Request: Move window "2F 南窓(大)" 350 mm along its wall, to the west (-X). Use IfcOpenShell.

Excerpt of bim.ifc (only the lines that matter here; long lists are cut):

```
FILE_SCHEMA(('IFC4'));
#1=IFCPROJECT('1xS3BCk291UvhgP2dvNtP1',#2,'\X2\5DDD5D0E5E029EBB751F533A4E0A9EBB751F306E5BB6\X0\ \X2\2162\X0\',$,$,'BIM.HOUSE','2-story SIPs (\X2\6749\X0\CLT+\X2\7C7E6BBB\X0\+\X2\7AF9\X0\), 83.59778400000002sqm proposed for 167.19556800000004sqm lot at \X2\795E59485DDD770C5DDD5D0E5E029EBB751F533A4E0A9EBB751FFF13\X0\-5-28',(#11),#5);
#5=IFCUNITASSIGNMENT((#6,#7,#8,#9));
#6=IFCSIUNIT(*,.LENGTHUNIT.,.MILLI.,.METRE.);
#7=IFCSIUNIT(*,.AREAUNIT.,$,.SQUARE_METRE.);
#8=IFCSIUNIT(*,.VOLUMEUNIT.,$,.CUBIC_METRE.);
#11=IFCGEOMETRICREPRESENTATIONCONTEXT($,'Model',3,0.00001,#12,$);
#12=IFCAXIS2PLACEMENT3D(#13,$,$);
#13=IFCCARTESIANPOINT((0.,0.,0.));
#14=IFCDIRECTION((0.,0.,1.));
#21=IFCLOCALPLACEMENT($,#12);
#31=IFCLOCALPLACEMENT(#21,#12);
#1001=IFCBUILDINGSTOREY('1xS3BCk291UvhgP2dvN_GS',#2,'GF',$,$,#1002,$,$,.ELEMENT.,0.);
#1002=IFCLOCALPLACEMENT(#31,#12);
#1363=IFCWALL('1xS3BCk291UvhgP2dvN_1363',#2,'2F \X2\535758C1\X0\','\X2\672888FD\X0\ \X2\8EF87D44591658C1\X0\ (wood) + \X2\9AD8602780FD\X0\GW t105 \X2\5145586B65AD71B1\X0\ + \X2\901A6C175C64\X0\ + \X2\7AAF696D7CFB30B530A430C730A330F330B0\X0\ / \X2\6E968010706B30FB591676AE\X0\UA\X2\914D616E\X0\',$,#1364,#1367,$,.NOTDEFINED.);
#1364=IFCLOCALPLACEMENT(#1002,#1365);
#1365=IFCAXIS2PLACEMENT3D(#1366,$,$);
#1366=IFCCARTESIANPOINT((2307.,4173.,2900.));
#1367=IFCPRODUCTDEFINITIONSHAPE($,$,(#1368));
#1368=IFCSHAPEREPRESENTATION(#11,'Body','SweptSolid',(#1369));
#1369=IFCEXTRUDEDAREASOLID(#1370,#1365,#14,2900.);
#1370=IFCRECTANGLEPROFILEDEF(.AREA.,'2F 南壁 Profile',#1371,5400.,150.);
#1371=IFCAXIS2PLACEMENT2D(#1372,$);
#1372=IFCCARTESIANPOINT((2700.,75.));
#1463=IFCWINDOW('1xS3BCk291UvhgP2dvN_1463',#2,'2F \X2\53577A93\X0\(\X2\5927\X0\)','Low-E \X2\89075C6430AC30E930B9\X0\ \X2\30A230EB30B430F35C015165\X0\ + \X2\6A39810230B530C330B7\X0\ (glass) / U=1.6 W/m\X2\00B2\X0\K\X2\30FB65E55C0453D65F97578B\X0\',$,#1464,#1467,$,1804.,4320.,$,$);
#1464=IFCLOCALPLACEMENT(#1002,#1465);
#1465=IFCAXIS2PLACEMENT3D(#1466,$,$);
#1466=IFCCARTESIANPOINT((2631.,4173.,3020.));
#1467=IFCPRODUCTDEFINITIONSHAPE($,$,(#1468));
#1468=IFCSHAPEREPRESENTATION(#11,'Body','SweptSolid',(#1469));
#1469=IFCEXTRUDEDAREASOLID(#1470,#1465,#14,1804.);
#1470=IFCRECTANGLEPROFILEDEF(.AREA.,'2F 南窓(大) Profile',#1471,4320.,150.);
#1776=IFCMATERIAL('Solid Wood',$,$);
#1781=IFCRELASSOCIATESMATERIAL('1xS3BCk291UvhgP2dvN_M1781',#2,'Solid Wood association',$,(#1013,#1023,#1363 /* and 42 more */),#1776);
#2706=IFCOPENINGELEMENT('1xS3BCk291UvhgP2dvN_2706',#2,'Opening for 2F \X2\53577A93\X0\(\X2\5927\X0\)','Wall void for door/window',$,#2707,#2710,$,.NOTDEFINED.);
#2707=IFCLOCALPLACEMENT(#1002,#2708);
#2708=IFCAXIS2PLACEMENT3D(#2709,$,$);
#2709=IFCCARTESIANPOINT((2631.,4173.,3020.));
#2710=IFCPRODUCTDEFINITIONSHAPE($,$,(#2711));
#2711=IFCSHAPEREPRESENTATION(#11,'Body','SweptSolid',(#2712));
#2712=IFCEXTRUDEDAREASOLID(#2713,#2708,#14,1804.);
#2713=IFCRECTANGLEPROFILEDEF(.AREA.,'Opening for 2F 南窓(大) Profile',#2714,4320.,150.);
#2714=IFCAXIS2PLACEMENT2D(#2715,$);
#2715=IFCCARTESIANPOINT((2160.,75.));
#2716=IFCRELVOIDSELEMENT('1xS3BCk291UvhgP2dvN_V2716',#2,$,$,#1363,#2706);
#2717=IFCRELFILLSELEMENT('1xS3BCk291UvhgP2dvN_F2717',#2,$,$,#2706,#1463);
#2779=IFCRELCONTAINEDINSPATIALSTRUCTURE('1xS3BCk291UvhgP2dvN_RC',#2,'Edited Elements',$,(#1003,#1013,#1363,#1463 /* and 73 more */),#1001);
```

```python
import ifcopenshell
import ifcopenshell.api.geometry
import ifcopenshell.util.placement

model = ifcopenshell.open("bim.ifc")

window = model.by_guid("1xS3BCk291UvhgP2dvN_1463")
opening = window.FillsVoids[0].RelatingOpeningElement
wall = opening.VoidsElements[0].RelatingBuildingElement

wall_matrix = ifcopenshell.util.placement.get_local_placement(wall.ObjectPlacement)
shift = wall_matrix[:3, 0] * -350.0
before = ifcopenshell.util.placement.get_local_placement(window.ObjectPlacement)[:3, 3].copy()

# The window is not placed relative to its opening, so move both.
for product in (opening, window):
    matrix = ifcopenshell.util.placement.get_local_placement(product.ObjectPlacement)
    matrix[:3, 3] += shift
    ifcopenshell.api.geometry.edit_object_placement(model, product=product, matrix=matrix, is_si=False)

after = ifcopenshell.util.placement.get_local_placement(window.ObjectPlacement)[:3, 3]
print("window moved by", (after - before).round(3) + 0.0)

model.write("bim-out.ifc")
```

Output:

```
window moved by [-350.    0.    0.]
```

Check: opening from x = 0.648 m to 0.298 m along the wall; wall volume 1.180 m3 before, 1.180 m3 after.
